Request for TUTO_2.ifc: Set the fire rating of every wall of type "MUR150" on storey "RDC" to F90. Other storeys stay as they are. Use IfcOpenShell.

First a look at what the model holds.

```python
import ifcopenshell
import ifcopenshell.util.element

model = ifcopenshell.open("TUTO_2.ifc")
print(model.schema)
storey = next(s for s in model.by_type("IfcBuildingStorey") if s.Name == "RDC")
walls = [e for e in ifcopenshell.util.element.get_decomposition(storey) if e.is_a("IfcWall")]
seen = {}
for e in walls:
    element_type = ifcopenshell.util.element.get_type(e)
    key = (element_type.Name if element_type != e and element_type else None, ifcopenshell.util.element.get_pset(e, "Pset_WallCommon", "FireRating"))
    seen[key] = seen.get(key, 0) + 1
for (name, value), count in sorted(seen.items(), key=str):
    print(count, "x", name, "|", value)
```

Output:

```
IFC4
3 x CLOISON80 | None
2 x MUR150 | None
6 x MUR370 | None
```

```python
import ifcopenshell
import ifcopenshell.api.pset
import ifcopenshell.util.element

model = ifcopenshell.open("TUTO_2.ifc")

storey = next(s for s in model.by_type("IfcBuildingStorey") if s.Name == "RDC")
walls = [e for e in ifcopenshell.util.element.get_decomposition(storey) if e.is_a("IfcWall")]

count = 0
for e in walls:
    element_type = ifcopenshell.util.element.get_type(e)
    if element_type in (None, e) or element_type.Name != "MUR150":
        continue
    # add_pset returns the element's existing set when there is one.
    pset = ifcopenshell.api.pset.add_pset(model, product=e, name="Pset_WallCommon")
    ifcopenshell.api.pset.edit_pset(model, pset=pset, properties={"FireRating": "F90"})
    count += 1

print(count, "walls updated")

model.write("TUTO_2_edited.ifc")
```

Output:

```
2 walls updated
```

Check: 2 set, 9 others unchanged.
